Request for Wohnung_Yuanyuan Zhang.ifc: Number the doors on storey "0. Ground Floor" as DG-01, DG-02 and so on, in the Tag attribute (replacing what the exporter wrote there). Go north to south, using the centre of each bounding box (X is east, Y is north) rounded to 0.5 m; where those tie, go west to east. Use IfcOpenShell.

First a look at what the model holds.

```python
import ifcopenshell
import ifcopenshell.util.element
import ifcopenshell.util.placement

model = ifcopenshell.open("Wohnung_Yuanyuan Zhang.ifc")
print(model.schema)
storey = next(s for s in model.by_type("IfcBuildingStorey") if s.Name == "0. Ground Floor")
doors = [e for e in ifcopenshell.util.element.get_decomposition(storey) if e.is_a("IfcDoor")]
for e in sorted(doors, key=lambda e: e.id()):
    origin = ifcopenshell.util.placement.get_local_placement(e.ObjectPlacement)[:3, 3]
    print(e.id(), e.Tag, e.Name, origin.round(2) + 0.0, sep=" | ")
```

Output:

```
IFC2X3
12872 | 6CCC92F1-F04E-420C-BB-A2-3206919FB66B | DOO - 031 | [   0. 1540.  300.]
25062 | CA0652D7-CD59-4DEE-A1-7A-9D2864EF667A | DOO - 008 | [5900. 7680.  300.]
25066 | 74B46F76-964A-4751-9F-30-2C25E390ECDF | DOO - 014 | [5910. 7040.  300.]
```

```python
import ifcopenshell
import ifcopenshell.geom
import ifcopenshell.util.element
import ifcopenshell.util.shape

model = ifcopenshell.open("Wohnung_Yuanyuan Zhang.ifc")
settings = ifcopenshell.geom.settings()
settings.set("use-world-coords", True)


def centre(element):
    shape = ifcopenshell.geom.create_shape(settings, element)
    return ifcopenshell.util.shape.get_bbox_centroid(shape.geometry)


storey = next(s for s in model.by_type("IfcBuildingStorey") if s.Name == "0. Ground Floor")
doors = [e for e in ifcopenshell.util.element.get_decomposition(storey) if e.is_a("IfcDoor")]

# Insertion points can sit at a corner or the storey origin, so sort by the geometry (in metres).
centres = {e: centre(e) for e in doors}
doors.sort(key=lambda e: (-round(centres[e][1] / 0.5), centres[e][0]))

for i, e in enumerate(doors, start=1):
    number = f"DG-{i:02d}"
    e.Tag = number
    print(e.id(), number)

model.write("Wohnung_Yuanyuan Zhang-out.ifc")
```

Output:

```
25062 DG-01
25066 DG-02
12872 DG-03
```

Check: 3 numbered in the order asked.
